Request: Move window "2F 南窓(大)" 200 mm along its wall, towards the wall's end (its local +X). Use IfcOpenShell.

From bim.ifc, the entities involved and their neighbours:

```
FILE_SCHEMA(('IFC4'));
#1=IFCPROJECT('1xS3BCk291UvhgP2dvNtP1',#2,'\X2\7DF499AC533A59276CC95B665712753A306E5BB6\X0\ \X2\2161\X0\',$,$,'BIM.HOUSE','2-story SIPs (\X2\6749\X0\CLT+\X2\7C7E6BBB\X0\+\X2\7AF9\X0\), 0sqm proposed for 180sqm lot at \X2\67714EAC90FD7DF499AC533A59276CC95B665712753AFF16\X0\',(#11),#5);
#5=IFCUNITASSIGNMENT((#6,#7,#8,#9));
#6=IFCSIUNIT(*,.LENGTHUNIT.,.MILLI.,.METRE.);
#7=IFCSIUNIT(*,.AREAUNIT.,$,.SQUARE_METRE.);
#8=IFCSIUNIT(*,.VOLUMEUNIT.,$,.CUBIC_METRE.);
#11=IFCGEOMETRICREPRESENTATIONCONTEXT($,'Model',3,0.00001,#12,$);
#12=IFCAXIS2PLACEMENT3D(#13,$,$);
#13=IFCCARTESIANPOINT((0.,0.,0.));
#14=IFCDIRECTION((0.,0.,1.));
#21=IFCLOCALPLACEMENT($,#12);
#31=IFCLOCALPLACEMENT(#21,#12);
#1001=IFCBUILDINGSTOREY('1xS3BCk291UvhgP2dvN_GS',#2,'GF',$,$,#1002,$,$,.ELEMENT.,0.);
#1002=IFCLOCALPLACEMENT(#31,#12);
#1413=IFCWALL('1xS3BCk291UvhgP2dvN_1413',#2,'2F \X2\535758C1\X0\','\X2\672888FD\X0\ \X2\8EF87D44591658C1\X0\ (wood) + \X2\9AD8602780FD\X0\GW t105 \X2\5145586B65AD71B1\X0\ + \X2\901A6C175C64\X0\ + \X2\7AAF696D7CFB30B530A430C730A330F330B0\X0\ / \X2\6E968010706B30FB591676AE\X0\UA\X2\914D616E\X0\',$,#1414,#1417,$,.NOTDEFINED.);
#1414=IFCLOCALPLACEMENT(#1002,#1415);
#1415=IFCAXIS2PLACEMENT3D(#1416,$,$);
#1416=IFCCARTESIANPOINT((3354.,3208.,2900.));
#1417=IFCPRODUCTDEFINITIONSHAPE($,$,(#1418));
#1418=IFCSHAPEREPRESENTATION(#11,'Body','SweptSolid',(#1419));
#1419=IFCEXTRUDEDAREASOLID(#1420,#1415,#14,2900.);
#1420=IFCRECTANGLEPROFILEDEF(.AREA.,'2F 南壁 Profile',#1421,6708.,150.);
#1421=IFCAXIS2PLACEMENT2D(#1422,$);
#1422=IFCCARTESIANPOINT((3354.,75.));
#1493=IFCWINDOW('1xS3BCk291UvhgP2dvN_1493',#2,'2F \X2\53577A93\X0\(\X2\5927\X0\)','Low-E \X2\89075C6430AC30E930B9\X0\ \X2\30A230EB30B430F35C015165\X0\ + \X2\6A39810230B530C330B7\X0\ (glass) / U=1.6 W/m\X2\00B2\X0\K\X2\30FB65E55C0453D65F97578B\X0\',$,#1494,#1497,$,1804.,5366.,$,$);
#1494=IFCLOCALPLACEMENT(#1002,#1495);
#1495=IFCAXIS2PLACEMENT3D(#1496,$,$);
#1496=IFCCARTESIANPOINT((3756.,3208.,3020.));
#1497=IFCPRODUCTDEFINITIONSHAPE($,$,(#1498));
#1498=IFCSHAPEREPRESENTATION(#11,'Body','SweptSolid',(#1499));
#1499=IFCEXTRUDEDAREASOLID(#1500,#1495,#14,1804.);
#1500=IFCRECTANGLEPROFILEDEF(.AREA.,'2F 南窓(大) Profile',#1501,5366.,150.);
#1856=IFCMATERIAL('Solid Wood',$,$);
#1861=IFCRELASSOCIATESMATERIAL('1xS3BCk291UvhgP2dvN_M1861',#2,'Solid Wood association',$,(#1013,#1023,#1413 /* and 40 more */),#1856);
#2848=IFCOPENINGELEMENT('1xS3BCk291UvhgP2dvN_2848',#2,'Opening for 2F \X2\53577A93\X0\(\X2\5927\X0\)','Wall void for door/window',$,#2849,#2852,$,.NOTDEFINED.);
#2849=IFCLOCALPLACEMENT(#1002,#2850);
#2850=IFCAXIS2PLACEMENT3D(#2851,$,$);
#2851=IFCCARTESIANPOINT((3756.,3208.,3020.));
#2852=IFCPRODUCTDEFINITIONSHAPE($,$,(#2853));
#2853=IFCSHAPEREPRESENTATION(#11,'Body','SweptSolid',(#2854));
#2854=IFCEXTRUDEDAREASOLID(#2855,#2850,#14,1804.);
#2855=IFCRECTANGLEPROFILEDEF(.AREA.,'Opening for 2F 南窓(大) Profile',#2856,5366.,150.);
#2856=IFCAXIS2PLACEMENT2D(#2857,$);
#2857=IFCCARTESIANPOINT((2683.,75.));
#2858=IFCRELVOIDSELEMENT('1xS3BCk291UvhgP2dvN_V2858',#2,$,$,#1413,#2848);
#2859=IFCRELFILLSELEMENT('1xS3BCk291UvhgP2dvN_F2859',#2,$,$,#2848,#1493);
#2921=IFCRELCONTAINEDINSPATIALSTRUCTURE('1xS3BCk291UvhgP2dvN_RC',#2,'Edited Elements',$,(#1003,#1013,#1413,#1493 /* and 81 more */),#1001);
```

```python
import ifcopenshell
import ifcopenshell.api.geometry
import ifcopenshell.util.placement

model = ifcopenshell.open("bim.ifc")

window = model.by_guid("1xS3BCk291UvhgP2dvN_1493")
opening = window.FillsVoids[0].RelatingOpeningElement
wall = opening.VoidsElements[0].RelatingBuildingElement

wall_matrix = ifcopenshell.util.placement.get_local_placement(wall.ObjectPlacement)
shift = wall_matrix[:3, 0] * 200.0
before = ifcopenshell.util.placement.get_local_placement(window.ObjectPlacement)[:3, 3].copy()

# The window is not placed relative to its opening, so move both.
for product in (opening, window):
    matrix = ifcopenshell.util.placement.get_local_placement(product.ObjectPlacement)
    matrix[:3, 3] += shift
    ifcopenshell.api.geometry.edit_object_placement(model, product=product, matrix=matrix, is_si=False)

after = ifcopenshell.util.placement.get_local_placement(window.ObjectPlacement)[:3, 3]
print("window moved by", (after - before).round(3) + 0.0)

model.write("bim_updated.ifc")
```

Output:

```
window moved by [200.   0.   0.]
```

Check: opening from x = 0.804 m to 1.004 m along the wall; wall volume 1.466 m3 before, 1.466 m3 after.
